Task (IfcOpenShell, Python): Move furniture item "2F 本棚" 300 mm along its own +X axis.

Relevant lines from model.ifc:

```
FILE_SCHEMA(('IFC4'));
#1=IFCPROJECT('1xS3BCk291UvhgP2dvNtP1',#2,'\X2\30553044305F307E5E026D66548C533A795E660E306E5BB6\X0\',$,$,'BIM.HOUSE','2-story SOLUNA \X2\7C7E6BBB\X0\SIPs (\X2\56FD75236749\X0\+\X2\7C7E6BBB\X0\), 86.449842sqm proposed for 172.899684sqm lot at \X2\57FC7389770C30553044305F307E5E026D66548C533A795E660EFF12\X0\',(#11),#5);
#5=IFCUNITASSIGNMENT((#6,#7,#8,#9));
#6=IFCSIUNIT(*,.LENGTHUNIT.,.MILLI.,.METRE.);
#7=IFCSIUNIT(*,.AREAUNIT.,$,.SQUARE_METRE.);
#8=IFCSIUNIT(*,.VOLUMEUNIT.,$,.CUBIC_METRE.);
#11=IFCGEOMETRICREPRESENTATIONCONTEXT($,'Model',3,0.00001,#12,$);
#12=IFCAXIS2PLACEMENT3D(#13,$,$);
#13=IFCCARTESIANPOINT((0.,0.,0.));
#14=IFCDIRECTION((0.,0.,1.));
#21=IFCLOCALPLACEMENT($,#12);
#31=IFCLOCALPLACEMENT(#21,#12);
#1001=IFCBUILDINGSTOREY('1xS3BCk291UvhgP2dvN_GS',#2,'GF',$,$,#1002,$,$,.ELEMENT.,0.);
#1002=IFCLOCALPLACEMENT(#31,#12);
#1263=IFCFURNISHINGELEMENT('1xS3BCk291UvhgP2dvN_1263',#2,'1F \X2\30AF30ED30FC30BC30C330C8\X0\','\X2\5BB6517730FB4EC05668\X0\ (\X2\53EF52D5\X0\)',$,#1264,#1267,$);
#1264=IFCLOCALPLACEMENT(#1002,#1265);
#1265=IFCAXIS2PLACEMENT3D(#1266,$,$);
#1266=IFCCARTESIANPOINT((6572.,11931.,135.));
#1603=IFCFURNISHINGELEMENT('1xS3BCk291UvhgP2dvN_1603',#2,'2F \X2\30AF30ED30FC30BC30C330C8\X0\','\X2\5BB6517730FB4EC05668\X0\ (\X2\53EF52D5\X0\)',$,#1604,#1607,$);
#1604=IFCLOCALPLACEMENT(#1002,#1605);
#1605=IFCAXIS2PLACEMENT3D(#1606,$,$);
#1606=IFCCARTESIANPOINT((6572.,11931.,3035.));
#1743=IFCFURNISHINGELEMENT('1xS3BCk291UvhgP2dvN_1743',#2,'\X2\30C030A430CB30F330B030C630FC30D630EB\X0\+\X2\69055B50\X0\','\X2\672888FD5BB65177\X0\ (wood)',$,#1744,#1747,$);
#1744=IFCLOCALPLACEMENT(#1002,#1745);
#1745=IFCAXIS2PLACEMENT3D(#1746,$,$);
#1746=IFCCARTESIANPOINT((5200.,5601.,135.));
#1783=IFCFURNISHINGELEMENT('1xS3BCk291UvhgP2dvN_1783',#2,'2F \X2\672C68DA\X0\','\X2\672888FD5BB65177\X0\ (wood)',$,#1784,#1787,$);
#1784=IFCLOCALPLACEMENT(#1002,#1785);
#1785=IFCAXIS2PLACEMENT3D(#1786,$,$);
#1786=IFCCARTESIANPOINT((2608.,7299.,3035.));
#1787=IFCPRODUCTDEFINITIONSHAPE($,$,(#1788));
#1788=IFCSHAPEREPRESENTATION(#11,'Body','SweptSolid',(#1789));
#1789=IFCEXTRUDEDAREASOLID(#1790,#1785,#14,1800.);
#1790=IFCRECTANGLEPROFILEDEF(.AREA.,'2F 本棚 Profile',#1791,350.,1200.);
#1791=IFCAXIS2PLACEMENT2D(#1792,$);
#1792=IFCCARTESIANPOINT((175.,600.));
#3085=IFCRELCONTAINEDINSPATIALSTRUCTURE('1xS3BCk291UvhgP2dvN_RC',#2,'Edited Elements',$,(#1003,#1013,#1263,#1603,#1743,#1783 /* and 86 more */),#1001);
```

```python
import ifcopenshell
import ifcopenshell.api.geometry
import ifcopenshell.util.placement
import ifcopenshell.util.unit

model = ifcopenshell.open("model.ifc")
unit_scale = ifcopenshell.util.unit.calculate_unit_scale(model)

item = model.by_id(1783)
matrix = ifcopenshell.util.placement.get_local_placement(item.ObjectPlacement)
matrix[:3, 3] += matrix[:3, 0] * 0.3 / unit_scale
ifcopenshell.api.geometry.edit_object_placement(model, product=item, matrix=matrix, is_si=False)

print(ifcopenshell.util.placement.get_local_placement(item.ObjectPlacement).round(3) + 0.0)

model.write("model-out.ifc")
```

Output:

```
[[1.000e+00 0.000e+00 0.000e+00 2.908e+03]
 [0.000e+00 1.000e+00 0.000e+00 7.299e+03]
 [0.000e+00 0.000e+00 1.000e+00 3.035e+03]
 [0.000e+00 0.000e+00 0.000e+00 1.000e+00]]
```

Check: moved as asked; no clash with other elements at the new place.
